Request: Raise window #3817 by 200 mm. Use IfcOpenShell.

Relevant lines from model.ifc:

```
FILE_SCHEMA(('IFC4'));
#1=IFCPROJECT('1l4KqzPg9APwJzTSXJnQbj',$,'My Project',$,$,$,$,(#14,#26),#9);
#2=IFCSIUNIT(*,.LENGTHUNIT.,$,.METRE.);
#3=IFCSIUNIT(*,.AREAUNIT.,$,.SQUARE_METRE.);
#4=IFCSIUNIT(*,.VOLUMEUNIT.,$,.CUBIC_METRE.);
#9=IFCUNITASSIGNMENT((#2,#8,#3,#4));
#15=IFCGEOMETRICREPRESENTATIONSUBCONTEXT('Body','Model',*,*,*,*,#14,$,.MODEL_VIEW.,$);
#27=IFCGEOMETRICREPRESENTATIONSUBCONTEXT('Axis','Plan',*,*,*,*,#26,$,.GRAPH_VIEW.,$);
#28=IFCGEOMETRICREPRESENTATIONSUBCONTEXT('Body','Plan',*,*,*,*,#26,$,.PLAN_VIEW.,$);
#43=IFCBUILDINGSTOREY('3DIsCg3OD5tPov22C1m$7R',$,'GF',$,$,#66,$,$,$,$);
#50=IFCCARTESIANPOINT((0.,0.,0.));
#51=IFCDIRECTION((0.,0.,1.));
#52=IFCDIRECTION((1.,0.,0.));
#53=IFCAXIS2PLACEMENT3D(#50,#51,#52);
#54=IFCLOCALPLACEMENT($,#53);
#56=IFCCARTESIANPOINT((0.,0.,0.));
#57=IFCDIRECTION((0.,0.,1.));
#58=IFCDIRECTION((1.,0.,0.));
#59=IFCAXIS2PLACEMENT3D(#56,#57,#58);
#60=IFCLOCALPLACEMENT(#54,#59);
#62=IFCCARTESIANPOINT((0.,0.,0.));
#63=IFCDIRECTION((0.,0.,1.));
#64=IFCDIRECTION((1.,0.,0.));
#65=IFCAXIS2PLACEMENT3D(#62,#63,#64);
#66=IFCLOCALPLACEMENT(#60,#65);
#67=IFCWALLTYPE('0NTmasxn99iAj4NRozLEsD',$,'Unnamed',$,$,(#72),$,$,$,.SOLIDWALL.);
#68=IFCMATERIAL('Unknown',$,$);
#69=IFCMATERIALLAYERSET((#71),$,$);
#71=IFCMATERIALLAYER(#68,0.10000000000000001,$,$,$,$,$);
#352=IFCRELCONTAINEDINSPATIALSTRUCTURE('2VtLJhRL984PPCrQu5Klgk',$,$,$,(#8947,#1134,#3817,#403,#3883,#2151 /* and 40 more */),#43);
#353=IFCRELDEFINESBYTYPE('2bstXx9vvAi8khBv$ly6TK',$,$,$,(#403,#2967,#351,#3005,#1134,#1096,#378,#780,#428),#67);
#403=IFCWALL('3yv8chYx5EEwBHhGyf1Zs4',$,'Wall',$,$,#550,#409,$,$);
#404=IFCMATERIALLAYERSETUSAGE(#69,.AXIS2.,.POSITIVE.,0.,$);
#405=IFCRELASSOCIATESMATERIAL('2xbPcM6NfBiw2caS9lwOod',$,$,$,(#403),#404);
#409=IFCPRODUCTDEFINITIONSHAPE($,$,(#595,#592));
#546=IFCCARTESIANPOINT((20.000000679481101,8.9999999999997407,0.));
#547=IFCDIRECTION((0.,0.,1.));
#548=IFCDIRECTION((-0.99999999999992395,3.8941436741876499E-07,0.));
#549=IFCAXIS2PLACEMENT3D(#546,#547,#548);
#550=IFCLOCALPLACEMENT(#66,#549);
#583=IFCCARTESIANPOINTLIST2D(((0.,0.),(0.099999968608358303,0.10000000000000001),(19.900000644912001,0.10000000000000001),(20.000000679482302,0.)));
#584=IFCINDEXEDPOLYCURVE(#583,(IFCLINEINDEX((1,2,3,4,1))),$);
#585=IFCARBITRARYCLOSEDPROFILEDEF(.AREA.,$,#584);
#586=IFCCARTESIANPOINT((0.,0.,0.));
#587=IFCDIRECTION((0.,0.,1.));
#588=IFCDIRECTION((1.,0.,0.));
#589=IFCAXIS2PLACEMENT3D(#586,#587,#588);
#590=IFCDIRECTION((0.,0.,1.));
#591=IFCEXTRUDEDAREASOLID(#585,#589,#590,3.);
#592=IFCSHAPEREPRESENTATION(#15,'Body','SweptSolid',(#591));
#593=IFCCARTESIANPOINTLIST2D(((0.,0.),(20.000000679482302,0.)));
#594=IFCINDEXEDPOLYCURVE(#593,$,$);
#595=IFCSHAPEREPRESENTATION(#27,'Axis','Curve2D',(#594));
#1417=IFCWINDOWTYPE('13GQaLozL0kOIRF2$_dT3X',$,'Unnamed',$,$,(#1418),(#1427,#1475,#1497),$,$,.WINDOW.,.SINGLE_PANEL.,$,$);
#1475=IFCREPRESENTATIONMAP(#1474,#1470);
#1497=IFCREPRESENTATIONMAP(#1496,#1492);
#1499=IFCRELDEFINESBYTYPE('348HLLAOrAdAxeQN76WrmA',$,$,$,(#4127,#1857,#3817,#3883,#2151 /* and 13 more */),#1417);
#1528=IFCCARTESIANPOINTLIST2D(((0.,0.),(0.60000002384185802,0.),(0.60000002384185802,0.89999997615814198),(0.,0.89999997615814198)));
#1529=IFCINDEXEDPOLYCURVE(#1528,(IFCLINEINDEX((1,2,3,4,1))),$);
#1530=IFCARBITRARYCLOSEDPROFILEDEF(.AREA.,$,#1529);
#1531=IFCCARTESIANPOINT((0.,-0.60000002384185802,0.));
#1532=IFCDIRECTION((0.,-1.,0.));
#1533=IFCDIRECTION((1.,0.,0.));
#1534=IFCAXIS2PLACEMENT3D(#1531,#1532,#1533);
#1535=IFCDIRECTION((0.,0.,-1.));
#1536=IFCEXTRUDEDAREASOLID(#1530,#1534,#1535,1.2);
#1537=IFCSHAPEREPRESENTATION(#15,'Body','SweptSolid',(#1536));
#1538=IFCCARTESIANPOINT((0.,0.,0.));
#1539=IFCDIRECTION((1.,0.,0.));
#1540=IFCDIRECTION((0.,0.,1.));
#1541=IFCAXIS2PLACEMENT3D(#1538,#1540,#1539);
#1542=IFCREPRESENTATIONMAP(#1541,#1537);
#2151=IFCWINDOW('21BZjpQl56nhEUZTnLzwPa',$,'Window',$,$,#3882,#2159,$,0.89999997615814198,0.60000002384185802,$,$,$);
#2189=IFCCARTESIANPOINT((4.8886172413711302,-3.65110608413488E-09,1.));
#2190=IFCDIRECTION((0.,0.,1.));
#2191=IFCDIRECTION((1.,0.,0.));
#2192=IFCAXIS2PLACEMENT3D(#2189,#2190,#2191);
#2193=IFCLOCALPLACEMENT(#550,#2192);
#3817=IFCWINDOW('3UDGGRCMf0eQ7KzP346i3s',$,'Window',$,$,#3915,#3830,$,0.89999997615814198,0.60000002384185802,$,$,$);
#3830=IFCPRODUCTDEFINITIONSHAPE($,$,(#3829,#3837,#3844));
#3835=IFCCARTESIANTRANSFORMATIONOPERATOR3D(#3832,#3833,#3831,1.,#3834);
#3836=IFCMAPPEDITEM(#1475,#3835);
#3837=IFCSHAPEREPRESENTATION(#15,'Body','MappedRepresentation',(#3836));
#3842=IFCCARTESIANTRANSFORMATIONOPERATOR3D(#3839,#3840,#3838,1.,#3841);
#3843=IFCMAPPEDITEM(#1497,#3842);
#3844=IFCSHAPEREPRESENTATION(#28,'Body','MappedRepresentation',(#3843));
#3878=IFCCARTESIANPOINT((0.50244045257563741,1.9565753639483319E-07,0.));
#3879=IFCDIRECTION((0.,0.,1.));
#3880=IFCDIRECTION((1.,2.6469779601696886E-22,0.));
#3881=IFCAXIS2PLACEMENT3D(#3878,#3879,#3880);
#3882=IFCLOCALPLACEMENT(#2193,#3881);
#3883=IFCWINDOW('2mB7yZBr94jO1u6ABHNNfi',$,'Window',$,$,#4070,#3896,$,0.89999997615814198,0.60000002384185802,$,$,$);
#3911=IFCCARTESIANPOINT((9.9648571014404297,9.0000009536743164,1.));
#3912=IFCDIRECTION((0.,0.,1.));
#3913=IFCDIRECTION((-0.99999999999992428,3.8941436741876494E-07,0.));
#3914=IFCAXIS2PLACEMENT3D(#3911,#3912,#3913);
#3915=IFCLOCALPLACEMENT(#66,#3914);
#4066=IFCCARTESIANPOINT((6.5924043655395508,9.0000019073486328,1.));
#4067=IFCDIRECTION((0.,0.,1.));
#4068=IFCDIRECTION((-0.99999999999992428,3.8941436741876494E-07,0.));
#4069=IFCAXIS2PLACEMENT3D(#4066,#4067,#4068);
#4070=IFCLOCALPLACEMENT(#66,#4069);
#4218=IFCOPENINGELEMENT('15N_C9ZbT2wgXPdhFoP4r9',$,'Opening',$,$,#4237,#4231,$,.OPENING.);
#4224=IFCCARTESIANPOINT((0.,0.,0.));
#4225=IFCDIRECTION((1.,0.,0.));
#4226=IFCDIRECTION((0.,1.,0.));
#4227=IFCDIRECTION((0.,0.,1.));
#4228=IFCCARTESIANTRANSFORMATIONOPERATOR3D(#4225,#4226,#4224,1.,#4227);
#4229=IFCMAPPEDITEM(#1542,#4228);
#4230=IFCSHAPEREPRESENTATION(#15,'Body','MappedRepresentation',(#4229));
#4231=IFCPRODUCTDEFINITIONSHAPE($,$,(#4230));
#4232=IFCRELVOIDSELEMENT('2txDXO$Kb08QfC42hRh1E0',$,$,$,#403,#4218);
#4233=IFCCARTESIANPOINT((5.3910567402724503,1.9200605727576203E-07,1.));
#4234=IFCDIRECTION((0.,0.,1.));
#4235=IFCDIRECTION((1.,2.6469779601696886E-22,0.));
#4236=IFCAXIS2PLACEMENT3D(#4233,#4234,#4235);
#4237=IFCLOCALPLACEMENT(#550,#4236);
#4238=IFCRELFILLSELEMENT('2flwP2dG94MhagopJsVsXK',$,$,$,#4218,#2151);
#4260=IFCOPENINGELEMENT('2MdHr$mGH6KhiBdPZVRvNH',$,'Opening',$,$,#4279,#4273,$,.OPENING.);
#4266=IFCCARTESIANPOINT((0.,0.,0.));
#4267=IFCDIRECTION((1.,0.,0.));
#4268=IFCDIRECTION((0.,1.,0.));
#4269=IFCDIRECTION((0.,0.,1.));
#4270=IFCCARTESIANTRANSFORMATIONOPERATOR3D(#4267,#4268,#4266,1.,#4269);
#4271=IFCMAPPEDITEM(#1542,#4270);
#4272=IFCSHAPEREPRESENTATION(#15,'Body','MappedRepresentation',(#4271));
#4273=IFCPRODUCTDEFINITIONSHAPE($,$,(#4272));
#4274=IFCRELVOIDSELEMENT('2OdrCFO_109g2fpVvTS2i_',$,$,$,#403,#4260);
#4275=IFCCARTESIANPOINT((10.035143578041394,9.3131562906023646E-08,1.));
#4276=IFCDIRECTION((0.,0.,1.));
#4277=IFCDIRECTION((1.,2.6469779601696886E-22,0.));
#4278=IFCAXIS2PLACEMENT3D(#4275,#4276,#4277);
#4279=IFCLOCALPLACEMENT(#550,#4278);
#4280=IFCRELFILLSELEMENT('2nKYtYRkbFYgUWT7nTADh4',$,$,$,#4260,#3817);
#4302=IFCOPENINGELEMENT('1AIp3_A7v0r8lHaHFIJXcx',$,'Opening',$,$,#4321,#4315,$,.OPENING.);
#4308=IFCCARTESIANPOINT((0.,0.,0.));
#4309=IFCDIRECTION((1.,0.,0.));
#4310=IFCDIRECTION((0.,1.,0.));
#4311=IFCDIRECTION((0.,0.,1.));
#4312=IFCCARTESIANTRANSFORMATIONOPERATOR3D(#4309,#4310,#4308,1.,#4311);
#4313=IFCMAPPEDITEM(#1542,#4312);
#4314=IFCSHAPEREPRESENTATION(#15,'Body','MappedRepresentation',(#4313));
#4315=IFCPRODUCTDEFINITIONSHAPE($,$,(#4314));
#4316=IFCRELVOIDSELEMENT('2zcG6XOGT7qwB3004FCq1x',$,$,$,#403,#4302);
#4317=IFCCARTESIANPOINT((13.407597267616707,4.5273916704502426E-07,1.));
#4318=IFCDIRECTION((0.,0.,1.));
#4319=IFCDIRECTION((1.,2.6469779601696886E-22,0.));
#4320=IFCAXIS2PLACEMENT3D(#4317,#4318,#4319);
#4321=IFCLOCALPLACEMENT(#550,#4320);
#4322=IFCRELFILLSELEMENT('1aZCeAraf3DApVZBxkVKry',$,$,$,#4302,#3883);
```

```python
import numpy as np
import ifcopenshell
import ifcopenshell.api.geometry
import ifcopenshell.util.placement
import ifcopenshell.util.unit

model = ifcopenshell.open("model.ifc")
unit_scale = ifcopenshell.util.unit.calculate_unit_scale(model)

window = model.by_id(3817)
opening = window.FillsVoids[0].RelatingOpeningElement
dz = 0.2 / unit_scale

shift = np.array([0.0, 0.0, dz])
# The window is not placed relative to its opening, so move both.
for product in (opening, window):
    matrix = ifcopenshell.util.placement.get_local_placement(product.ObjectPlacement)
    matrix[:3, 3] += shift
    ifcopenshell.api.geometry.edit_object_placement(model, product=product, matrix=matrix, is_si=False)

print(f"moved by {dz * unit_scale:+.3f} m")

model.write("model_edited.ifc")
```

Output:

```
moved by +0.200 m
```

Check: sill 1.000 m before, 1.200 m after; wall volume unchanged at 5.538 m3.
